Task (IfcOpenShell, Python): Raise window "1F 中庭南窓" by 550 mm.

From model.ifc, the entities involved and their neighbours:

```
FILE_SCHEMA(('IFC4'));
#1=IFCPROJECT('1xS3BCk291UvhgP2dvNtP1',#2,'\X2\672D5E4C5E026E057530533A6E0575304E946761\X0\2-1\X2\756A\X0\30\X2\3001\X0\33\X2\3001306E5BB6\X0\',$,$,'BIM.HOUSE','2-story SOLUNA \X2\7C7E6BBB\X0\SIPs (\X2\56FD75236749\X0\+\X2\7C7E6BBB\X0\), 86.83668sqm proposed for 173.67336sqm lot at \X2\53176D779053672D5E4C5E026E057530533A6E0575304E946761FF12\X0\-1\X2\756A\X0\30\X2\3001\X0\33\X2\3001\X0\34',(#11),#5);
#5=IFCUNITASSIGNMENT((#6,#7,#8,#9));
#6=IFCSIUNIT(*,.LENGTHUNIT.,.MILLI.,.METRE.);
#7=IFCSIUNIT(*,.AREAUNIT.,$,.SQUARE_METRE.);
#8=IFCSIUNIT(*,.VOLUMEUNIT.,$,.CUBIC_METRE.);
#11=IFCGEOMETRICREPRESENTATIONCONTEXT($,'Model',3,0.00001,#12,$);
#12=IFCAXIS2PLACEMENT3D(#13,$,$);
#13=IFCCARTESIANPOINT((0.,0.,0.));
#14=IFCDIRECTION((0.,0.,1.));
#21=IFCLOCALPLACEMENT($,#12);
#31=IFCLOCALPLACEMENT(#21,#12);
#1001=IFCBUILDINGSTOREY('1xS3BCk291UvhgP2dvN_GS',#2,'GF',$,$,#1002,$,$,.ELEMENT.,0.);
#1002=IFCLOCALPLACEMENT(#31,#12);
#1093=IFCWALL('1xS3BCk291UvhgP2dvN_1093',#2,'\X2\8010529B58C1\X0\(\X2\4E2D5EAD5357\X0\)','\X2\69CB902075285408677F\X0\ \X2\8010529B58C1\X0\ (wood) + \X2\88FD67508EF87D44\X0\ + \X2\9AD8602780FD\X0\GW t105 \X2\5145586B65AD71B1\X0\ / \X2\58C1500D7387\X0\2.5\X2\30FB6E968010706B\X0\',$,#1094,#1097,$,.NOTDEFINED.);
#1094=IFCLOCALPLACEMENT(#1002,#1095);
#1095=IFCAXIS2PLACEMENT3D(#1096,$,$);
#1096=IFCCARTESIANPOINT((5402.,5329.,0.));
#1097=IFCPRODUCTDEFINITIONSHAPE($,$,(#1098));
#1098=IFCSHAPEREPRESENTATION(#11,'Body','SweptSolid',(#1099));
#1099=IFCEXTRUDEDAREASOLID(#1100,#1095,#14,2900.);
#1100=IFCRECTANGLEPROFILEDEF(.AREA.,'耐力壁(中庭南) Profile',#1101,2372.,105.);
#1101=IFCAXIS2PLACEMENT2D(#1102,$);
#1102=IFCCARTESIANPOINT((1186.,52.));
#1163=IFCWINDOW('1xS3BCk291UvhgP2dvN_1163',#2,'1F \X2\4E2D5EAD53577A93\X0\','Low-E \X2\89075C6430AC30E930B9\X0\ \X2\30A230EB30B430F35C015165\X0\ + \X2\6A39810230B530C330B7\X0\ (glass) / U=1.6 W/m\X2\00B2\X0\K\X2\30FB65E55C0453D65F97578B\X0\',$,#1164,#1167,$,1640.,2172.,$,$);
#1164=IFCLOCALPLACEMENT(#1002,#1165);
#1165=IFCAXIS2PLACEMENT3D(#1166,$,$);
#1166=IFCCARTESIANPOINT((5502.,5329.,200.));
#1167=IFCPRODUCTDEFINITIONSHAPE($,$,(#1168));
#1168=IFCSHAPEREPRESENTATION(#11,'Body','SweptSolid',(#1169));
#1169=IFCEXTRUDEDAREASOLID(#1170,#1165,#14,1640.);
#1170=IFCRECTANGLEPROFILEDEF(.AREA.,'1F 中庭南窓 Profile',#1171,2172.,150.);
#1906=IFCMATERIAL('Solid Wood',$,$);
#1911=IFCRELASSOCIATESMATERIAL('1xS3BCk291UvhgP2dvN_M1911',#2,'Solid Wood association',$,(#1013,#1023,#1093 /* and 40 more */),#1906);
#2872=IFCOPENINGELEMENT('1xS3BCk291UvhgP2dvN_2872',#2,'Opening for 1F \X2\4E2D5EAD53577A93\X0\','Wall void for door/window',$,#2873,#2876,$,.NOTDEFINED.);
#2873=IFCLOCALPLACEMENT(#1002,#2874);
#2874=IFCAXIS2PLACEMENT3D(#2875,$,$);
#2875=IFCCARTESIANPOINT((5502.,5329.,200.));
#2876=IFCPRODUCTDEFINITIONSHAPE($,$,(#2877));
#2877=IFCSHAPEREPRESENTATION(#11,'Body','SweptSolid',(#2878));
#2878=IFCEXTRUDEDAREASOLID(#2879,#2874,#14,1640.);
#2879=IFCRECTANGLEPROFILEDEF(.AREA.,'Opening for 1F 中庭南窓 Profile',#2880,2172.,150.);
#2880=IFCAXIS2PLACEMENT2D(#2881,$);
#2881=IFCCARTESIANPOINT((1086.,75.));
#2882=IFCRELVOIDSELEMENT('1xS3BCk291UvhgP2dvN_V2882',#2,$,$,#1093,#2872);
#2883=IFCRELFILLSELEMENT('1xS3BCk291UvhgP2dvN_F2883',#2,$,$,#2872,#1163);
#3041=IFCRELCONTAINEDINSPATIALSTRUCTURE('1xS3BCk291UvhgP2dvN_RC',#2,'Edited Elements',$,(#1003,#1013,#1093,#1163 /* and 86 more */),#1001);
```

```python
import numpy as np
import ifcopenshell
import ifcopenshell.api.geometry
import ifcopenshell.util.placement
import ifcopenshell.util.unit

model = ifcopenshell.open("model.ifc")
unit_scale = ifcopenshell.util.unit.calculate_unit_scale(model)

window = model.by_id(1163)
opening = window.FillsVoids[0].RelatingOpeningElement
dz = 0.55 / unit_scale

shift = np.array([0.0, 0.0, dz])
# The window is not placed relative to its opening, so move both.
for product in (opening, window):
    matrix = ifcopenshell.util.placement.get_local_placement(product.ObjectPlacement)
    matrix[:3, 3] += shift
    ifcopenshell.api.geometry.edit_object_placement(model, product=product, matrix=matrix, is_si=False)

print(f"moved by {dz * unit_scale:+.3f} m")

model.write("model_updated.ifc")
```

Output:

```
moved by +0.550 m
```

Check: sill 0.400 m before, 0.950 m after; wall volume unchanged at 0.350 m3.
